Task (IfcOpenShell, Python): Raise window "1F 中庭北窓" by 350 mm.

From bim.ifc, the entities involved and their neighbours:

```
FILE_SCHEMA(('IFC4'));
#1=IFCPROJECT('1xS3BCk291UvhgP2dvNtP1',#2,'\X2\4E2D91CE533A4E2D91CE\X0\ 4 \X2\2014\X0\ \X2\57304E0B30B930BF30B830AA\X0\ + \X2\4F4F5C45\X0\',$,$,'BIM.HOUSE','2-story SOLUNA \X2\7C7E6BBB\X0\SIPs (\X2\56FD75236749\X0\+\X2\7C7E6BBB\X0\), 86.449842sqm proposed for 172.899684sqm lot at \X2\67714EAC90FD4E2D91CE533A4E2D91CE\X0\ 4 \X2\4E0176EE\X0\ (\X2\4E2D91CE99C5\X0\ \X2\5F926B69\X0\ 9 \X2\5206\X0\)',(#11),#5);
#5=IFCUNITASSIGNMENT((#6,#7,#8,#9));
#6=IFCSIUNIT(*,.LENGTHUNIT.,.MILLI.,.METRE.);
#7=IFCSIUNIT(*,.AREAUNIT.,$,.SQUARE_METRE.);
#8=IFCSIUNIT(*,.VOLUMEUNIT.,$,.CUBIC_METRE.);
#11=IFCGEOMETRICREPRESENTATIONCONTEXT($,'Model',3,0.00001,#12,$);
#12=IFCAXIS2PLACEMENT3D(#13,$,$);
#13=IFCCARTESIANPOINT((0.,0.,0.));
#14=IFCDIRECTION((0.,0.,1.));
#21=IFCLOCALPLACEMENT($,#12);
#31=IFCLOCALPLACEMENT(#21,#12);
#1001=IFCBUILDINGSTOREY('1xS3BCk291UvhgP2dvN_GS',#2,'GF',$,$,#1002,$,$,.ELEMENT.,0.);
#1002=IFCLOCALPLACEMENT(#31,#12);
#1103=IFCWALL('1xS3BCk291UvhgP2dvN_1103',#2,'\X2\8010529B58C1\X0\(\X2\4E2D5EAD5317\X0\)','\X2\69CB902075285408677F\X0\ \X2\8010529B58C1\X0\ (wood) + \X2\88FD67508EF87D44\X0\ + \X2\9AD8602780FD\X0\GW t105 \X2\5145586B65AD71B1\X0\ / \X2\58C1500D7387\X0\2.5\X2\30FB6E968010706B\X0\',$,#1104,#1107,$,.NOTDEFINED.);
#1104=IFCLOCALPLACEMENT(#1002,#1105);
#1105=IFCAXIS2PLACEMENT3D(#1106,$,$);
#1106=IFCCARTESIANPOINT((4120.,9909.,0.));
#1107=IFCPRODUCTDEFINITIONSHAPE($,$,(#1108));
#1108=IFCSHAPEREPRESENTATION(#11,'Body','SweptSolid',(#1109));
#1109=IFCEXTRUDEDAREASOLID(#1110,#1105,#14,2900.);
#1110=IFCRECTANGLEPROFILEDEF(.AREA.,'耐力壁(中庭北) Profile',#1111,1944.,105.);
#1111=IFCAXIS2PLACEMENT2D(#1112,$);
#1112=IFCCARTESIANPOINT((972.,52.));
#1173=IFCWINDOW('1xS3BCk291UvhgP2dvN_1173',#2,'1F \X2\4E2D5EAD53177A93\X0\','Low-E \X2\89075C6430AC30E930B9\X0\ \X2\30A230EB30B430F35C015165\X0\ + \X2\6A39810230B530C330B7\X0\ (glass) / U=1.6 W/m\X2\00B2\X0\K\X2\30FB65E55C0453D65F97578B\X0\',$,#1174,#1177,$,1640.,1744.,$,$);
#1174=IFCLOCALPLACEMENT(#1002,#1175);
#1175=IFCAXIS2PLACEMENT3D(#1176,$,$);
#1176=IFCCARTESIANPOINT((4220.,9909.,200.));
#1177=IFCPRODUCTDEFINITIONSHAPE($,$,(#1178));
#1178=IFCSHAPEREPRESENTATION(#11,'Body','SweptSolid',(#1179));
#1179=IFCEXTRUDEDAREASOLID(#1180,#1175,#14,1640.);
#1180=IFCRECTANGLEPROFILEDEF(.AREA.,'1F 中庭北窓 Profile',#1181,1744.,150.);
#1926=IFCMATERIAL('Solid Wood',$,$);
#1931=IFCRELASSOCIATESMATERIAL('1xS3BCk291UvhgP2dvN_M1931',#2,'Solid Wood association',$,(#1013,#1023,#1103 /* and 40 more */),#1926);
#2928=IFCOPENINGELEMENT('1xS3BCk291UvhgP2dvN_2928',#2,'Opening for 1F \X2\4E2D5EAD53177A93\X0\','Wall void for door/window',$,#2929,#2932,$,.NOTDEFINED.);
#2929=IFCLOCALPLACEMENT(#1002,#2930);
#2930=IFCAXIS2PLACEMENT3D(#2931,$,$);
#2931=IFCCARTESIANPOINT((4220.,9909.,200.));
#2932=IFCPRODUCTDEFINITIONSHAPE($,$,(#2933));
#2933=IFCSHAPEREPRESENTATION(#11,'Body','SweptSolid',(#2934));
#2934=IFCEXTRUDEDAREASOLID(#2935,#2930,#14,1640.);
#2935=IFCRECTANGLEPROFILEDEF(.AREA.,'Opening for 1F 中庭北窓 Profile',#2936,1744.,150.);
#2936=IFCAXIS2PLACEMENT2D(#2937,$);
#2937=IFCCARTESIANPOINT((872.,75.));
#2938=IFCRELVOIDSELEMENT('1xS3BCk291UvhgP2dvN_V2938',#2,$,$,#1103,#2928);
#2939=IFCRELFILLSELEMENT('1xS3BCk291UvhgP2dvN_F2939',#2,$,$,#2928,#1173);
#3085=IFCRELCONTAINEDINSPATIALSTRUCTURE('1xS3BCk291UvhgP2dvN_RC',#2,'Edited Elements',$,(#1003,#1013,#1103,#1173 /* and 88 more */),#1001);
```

```python
import numpy as np
import ifcopenshell
import ifcopenshell.api.geometry
import ifcopenshell.util.placement
import ifcopenshell.util.unit

model = ifcopenshell.open("bim.ifc")
unit_scale = ifcopenshell.util.unit.calculate_unit_scale(model)

window = model.by_guid("1xS3BCk291UvhgP2dvN_1173")
opening = window.FillsVoids[0].RelatingOpeningElement
dz = 0.35 / unit_scale

shift = np.array([0.0, 0.0, dz])
# The window is not placed relative to its opening, so move both.
for product in (opening, window):
    matrix = ifcopenshell.util.placement.get_local_placement(product.ObjectPlacement)
    matrix[:3, 3] += shift
    ifcopenshell.api.geometry.edit_object_placement(model, product=product, matrix=matrix, is_si=False)

print(f"moved by {dz * unit_scale:+.3f} m")

model.write("bim_v2.ifc")
```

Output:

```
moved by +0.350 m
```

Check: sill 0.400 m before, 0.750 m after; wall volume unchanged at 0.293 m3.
